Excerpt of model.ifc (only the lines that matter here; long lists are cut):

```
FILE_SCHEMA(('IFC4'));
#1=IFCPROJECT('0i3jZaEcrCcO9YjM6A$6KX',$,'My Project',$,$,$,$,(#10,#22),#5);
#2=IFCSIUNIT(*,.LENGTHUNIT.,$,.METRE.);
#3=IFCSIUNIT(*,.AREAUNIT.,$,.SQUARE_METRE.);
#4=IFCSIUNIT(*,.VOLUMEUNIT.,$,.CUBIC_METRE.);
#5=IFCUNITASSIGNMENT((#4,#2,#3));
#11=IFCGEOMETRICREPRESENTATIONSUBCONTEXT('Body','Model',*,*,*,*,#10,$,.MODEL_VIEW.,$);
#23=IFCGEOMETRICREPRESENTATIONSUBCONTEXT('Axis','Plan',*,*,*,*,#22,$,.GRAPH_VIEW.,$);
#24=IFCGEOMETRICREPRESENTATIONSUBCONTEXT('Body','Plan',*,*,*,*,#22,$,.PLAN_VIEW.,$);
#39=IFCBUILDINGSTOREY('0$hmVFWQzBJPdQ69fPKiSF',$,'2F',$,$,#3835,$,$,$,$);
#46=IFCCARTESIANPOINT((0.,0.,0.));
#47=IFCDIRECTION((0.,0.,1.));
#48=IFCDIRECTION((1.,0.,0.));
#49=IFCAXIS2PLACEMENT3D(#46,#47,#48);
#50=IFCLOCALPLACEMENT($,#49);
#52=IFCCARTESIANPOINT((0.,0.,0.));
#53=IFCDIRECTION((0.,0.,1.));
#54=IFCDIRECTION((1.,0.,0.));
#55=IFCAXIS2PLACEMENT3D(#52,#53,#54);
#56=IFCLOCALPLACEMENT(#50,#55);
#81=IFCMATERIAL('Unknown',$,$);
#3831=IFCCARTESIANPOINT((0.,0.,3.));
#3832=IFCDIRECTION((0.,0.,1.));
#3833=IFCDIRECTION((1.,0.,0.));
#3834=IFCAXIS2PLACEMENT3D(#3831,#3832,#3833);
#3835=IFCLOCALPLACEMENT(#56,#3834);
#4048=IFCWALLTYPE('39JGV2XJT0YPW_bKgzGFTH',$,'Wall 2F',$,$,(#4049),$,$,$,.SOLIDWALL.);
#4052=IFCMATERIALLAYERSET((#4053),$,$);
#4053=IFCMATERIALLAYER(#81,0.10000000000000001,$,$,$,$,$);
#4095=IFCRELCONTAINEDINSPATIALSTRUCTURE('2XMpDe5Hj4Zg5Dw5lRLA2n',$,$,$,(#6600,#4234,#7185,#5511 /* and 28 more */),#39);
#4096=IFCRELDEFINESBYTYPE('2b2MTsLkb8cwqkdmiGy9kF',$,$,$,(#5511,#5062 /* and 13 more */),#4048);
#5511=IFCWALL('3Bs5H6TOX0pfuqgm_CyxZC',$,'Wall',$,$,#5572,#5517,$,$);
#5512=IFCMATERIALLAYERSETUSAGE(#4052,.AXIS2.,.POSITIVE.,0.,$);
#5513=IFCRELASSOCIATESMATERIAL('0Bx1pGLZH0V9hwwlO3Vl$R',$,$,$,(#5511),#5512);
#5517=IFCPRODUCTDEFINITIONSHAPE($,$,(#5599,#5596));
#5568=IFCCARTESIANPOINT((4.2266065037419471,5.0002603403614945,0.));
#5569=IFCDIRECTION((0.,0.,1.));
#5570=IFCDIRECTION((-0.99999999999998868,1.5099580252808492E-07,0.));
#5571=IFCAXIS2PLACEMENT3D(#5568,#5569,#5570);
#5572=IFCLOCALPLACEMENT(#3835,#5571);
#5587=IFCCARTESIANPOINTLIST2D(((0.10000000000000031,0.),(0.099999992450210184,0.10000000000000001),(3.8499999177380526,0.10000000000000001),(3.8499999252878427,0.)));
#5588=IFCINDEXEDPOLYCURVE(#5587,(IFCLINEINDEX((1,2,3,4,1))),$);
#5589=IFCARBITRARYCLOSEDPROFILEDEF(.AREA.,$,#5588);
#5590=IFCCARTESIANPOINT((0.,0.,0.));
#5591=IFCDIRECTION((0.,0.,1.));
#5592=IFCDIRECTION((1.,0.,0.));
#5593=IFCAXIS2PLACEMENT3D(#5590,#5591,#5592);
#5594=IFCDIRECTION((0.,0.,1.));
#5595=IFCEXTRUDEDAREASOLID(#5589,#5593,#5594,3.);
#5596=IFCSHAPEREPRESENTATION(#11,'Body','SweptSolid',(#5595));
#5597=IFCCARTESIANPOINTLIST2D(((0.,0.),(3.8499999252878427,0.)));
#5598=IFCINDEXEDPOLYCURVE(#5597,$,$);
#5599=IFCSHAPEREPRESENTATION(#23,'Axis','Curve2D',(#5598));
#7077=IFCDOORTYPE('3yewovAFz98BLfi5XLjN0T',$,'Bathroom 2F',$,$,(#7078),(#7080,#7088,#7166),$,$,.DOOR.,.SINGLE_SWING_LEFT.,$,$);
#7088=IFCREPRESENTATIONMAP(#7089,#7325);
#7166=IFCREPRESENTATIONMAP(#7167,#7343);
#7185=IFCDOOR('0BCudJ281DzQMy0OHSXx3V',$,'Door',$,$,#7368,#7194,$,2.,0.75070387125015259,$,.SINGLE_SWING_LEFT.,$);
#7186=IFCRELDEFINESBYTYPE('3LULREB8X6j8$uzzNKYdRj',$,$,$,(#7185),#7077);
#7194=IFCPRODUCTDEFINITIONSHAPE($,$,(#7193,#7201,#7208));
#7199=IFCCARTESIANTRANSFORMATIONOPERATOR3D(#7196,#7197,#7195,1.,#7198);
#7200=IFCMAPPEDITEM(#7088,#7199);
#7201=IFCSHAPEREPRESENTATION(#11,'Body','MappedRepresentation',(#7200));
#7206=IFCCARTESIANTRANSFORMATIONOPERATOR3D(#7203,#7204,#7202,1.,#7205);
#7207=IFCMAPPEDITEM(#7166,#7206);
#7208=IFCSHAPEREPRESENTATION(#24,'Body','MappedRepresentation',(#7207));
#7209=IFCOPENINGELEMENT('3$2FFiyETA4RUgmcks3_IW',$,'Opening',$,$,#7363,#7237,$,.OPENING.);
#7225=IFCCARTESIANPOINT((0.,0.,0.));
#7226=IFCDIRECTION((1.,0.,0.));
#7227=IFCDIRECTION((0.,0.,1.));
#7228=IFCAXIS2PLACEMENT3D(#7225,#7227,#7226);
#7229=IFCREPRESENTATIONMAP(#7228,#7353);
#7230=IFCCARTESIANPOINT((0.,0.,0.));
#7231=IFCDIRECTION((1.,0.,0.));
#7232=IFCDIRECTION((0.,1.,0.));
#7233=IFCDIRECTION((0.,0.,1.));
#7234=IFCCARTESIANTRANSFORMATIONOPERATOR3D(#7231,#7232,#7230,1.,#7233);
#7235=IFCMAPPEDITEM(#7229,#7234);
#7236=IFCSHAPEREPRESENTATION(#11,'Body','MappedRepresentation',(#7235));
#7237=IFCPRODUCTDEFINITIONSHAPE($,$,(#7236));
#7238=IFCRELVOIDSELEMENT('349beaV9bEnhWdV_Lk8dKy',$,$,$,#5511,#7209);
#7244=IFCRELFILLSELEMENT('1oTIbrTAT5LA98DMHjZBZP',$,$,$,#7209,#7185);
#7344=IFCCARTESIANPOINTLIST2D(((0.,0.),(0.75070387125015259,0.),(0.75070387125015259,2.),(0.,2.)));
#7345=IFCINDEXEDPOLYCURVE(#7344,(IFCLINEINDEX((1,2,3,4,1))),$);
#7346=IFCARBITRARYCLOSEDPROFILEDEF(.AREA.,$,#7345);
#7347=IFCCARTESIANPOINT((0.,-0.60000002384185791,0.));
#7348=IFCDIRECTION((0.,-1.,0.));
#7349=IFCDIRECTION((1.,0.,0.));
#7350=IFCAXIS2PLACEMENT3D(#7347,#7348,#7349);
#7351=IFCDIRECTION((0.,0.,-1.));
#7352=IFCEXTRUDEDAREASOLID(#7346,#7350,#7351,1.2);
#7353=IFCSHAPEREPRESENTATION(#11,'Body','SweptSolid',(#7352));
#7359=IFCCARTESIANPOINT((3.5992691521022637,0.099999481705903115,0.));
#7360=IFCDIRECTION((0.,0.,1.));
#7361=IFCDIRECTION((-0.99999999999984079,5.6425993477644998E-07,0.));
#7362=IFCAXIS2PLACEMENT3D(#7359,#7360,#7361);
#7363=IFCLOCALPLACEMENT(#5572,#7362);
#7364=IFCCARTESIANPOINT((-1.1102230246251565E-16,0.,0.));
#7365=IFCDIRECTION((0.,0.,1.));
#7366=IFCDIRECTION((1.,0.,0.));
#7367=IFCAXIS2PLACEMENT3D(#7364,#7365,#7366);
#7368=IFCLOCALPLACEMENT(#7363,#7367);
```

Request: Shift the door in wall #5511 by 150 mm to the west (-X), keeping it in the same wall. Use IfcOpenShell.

```python
import ifcopenshell
import ifcopenshell.api.geometry
import ifcopenshell.util.placement
import ifcopenshell.util.unit

model = ifcopenshell.open("model.ifc")
unit_scale = ifcopenshell.util.unit.calculate_unit_scale(model)

door = model.by_guid("0BCudJ281DzQMy0OHSXx3V")
opening = door.FillsVoids[0].RelatingOpeningElement
wall = opening.VoidsElements[0].RelatingBuildingElement

wall_matrix = ifcopenshell.util.placement.get_local_placement(wall.ObjectPlacement)
shift = wall_matrix[:3, 0] * 0.15 / unit_scale
before = ifcopenshell.util.placement.get_local_placement(door.ObjectPlacement)[:3, 3].copy()

# The door is placed relative to its opening, so it follows when the opening moves.
matrix = ifcopenshell.util.placement.get_local_placement(opening.ObjectPlacement)
matrix[:3, 3] += shift
ifcopenshell.api.geometry.edit_object_placement(
    model, product=opening, matrix=matrix, is_si=False, should_transform_children=True
)

after = ifcopenshell.util.placement.get_local_placement(door.ObjectPlacement)[:3, 3]
print("door moved by", (after - before).round(3) + 0.0)

model.write("model_v2.ifc")
```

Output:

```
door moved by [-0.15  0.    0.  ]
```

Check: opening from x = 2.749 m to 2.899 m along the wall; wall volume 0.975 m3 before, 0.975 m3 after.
